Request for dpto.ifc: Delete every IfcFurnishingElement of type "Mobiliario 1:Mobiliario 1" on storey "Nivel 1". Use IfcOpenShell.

First a look at what the model holds.

```python
import ifcopenshell
import ifcopenshell.util.element

model = ifcopenshell.open("dpto.ifc")
print(model.schema)
storey = next(s for s in model.by_type("IfcBuildingStorey") if s.Name == "Nivel 1")
furniture = [e for e in ifcopenshell.util.element.get_decomposition(storey) if e.is_a("IfcFurnishingElement")]
seen = {}
for e in furniture:
    element_type = ifcopenshell.util.element.get_type(e)
    name = element_type.Name if element_type not in (None, e) else None
    seen[name] = seen.get(name, 0) + 1
for name, count in sorted(seen.items(), key=str):
    print(count, "x", name)
```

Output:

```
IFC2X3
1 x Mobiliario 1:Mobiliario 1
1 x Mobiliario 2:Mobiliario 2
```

```python
import ifcopenshell
import ifcopenshell.api.root
import ifcopenshell.util.element

model = ifcopenshell.open("dpto.ifc")

storey = next(s for s in model.by_type("IfcBuildingStorey") if s.Name == "Nivel 1")
furniture = [e for e in ifcopenshell.util.element.get_decomposition(storey) if e.is_a("IfcFurnishingElement")]
targets = [e for e in furniture if (t := ifcopenshell.util.element.get_type(e)) not in (None, e) and t.Name == "Mobiliario 1:Mobiliario 1"]

for e in targets:
    ifcopenshell.api.root.remove_product(model, product=e)
print(len(targets), "removed")

model.write("dpto_v2.ifc")
```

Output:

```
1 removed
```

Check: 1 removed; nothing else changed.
